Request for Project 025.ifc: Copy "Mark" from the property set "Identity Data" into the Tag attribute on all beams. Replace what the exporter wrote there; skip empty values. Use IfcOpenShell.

First a look at what the model holds.

```python
import ifcopenshell
import ifcopenshell.util.element

model = ifcopenshell.open("Project 025.ifc")
print(model.schema)
beams = model.by_type("IfcBeam")
print(len(beams), "beams")
for e in beams[:8]:
    source = ifcopenshell.util.element.get_pset(e, "Identity Data", "Mark")
    target = e.Tag
    print(e.id(), repr(source), repr(target), sep=" | ")
```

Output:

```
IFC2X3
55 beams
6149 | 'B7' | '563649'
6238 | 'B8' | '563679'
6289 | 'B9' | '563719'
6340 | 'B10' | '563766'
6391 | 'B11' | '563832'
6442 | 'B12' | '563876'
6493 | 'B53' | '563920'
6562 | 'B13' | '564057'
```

```python
import ifcopenshell
import ifcopenshell.util.element

model = ifcopenshell.open("Project 025.ifc")

count = 0
for e in model.by_type("IfcBeam"):
    value = ifcopenshell.util.element.get_pset(e, "Identity Data", "Mark")
    current = e.Tag
    if not value or not value.strip() or current == value:
        continue
    e.Tag = value
    count += 1

print(count, "beams updated")

model.write("Project 025_v2.ifc")
```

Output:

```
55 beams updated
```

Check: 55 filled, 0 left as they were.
